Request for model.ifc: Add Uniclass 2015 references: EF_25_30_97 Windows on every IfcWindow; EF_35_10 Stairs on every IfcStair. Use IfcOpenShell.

First a look at what the model holds.

```python
import ifcopenshell

model = ifcopenshell.open("model.ifc")
print(model.schema)
print("classifications:", [c.Name for c in model.by_type("IfcClassification")])
for ifc_class in ("IfcDoor", "IfcRoof", "IfcStair", "IfcWall", "IfcWindow"):
    print(ifc_class, len(model.by_type(ifc_class)))
```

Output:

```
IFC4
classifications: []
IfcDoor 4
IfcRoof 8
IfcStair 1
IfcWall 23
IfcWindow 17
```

```python
import ifcopenshell
import ifcopenshell.api.classification

model = ifcopenshell.open("model.ifc")

system = ifcopenshell.api.classification.add_classification(model, classification="Uniclass 2015")

codes = {
    "IfcWindow": ("EF_25_30_97", "Windows"),
    "IfcStair": ("EF_35_10", "Stairs"),
}
for ifc_class, (code, name) in codes.items():
    products = model.by_type(ifc_class)
    ifcopenshell.api.classification.add_reference(
        model, products=products, classification=system, identification=code, name=name
    )
    print(code, len(products))

model.write("model_rev.ifc")
```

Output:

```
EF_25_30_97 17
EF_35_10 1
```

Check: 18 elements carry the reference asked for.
